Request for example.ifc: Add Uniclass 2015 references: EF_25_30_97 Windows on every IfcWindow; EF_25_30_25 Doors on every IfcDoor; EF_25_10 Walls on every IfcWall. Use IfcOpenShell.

First a look at what the model holds.

```python
import ifcopenshell

model = ifcopenshell.open("example.ifc")
print(model.schema)
print("classifications:", [c.Name for c in model.by_type("IfcClassification")])
for ifc_class in ("IfcDoor", "IfcRoof", "IfcStair", "IfcWall", "IfcWindow"):
    print(ifc_class, len(model.by_type(ifc_class)))
```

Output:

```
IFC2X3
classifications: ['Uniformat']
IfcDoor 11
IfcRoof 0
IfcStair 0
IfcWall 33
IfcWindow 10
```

```python
import ifcopenshell
import ifcopenshell.api.classification

model = ifcopenshell.open("example.ifc")

# IFC2X3 requires Source and Edition and has no link from the project to the system.
system = model.create_entity("IfcClassification", Source="NBS", Edition="2015", Name="Uniclass 2015")

codes = {
    "IfcWindow": ("EF_25_30_97", "Windows"),
    "IfcDoor": ("EF_25_30_25", "Doors"),
    "IfcWall": ("EF_25_10", "Walls"),
}
for ifc_class, (code, name) in codes.items():
    products = model.by_type(ifc_class)
    ifcopenshell.api.classification.add_reference(
        model, products=products, classification=system, identification=code, name=name
    )
    print(code, len(products))

model.write("example_v2.ifc")
```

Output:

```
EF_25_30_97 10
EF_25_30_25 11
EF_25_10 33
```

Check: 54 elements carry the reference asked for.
